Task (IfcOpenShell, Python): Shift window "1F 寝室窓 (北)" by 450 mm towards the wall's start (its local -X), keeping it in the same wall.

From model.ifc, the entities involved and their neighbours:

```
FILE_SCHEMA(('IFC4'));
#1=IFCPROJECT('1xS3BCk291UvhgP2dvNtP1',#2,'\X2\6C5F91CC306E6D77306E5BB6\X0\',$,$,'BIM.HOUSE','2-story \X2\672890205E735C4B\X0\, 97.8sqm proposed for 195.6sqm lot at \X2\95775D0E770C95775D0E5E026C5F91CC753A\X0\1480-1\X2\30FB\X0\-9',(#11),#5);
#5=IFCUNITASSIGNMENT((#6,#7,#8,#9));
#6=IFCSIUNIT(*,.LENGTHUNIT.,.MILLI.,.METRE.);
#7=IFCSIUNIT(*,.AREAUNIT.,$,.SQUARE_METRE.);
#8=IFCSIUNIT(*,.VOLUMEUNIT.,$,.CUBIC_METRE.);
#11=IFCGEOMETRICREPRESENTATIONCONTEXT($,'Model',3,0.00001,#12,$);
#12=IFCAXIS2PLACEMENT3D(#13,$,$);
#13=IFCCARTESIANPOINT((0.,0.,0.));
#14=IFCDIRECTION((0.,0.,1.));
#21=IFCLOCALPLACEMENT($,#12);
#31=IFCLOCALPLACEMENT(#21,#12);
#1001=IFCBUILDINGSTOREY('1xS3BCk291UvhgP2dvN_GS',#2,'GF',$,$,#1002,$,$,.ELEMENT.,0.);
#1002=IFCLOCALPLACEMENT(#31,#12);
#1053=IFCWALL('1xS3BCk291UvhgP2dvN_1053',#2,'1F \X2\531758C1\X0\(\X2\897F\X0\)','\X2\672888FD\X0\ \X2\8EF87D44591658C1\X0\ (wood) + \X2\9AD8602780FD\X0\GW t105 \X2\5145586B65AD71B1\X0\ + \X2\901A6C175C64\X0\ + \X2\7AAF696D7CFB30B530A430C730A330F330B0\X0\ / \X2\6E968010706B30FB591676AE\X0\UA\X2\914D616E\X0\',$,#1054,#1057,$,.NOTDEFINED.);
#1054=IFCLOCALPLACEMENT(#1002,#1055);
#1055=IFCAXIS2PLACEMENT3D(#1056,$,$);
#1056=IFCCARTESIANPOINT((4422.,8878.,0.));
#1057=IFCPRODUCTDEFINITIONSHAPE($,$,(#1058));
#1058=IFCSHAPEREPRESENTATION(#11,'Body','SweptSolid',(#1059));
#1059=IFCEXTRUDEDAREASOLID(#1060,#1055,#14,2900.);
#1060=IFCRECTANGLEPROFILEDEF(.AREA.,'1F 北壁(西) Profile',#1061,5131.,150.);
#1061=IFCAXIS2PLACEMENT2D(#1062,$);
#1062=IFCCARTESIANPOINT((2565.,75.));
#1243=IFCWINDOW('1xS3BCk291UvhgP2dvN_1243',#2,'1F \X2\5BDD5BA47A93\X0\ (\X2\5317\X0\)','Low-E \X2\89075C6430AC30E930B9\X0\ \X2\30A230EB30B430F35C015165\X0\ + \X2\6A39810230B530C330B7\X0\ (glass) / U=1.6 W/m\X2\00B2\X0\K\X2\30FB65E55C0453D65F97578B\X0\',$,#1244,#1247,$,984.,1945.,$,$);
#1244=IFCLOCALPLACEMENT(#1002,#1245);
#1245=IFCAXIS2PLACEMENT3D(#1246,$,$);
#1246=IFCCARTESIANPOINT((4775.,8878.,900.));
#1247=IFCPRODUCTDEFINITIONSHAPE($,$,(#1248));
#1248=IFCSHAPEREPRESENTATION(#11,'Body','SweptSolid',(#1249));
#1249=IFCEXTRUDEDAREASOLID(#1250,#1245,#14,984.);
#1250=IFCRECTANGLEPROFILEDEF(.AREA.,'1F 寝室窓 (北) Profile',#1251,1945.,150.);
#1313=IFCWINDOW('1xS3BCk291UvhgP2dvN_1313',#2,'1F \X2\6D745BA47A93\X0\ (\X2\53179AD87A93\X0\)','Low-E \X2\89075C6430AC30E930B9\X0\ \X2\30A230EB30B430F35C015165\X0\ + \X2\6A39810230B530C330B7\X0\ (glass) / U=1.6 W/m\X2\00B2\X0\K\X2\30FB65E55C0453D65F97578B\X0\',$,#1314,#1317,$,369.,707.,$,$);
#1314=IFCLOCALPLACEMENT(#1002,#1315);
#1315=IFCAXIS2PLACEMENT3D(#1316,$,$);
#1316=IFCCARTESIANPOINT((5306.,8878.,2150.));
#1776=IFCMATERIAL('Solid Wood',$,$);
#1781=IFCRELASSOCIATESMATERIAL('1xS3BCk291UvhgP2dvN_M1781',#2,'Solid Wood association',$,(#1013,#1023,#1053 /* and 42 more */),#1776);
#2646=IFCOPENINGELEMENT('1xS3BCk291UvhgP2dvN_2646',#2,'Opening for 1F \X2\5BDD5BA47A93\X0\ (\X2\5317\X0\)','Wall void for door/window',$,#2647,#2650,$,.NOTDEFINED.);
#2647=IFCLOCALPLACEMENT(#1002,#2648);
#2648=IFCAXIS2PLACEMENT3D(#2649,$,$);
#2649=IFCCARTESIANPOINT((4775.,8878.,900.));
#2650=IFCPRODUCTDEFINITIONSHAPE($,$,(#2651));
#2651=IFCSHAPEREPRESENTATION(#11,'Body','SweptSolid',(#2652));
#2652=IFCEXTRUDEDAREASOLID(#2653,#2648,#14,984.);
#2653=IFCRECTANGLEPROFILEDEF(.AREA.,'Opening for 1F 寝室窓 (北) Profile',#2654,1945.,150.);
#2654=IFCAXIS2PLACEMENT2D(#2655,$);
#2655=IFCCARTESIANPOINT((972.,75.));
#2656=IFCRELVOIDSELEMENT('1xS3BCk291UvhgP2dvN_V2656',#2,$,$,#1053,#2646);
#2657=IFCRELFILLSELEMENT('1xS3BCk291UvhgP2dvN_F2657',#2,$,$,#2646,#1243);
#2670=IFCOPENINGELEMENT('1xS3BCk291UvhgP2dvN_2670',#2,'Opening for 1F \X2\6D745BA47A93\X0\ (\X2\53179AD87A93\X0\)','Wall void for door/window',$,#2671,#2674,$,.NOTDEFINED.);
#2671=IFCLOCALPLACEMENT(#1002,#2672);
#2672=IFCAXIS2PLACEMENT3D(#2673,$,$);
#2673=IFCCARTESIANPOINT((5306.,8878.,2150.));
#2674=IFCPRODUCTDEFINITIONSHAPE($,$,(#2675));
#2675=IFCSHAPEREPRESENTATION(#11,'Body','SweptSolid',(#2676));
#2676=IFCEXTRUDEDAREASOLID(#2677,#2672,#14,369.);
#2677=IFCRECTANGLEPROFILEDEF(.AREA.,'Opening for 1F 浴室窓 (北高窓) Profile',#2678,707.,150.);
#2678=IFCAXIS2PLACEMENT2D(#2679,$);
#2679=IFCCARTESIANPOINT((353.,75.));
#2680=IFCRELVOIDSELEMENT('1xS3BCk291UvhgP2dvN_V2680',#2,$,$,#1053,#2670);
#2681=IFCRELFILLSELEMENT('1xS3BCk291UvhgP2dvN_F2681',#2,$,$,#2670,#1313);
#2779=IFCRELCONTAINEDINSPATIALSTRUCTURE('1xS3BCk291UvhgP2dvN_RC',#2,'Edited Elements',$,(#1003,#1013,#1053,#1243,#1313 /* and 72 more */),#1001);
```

```python
import ifcopenshell
import ifcopenshell.api.geometry
import ifcopenshell.util.placement

model = ifcopenshell.open("model.ifc")

window = model.by_id(1243)
opening = window.FillsVoids[0].RelatingOpeningElement
wall = opening.VoidsElements[0].RelatingBuildingElement

wall_matrix = ifcopenshell.util.placement.get_local_placement(wall.ObjectPlacement)
shift = wall_matrix[:3, 0] * -450.0
before = ifcopenshell.util.placement.get_local_placement(window.ObjectPlacement)[:3, 3].copy()

# The window is not placed relative to its opening, so move both.
for product in (opening, window):
    matrix = ifcopenshell.util.placement.get_local_placement(product.ObjectPlacement)
    matrix[:3, 3] += shift
    ifcopenshell.api.geometry.edit_object_placement(model, product=product, matrix=matrix, is_si=False)

after = ifcopenshell.util.placement.get_local_placement(window.ObjectPlacement)[:3, 3]
print("window moved by", (after - before).round(3) + 0.0)

model.write("model_updated.ifc")
```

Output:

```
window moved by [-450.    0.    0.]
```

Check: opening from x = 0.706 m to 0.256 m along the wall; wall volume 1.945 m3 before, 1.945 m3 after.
